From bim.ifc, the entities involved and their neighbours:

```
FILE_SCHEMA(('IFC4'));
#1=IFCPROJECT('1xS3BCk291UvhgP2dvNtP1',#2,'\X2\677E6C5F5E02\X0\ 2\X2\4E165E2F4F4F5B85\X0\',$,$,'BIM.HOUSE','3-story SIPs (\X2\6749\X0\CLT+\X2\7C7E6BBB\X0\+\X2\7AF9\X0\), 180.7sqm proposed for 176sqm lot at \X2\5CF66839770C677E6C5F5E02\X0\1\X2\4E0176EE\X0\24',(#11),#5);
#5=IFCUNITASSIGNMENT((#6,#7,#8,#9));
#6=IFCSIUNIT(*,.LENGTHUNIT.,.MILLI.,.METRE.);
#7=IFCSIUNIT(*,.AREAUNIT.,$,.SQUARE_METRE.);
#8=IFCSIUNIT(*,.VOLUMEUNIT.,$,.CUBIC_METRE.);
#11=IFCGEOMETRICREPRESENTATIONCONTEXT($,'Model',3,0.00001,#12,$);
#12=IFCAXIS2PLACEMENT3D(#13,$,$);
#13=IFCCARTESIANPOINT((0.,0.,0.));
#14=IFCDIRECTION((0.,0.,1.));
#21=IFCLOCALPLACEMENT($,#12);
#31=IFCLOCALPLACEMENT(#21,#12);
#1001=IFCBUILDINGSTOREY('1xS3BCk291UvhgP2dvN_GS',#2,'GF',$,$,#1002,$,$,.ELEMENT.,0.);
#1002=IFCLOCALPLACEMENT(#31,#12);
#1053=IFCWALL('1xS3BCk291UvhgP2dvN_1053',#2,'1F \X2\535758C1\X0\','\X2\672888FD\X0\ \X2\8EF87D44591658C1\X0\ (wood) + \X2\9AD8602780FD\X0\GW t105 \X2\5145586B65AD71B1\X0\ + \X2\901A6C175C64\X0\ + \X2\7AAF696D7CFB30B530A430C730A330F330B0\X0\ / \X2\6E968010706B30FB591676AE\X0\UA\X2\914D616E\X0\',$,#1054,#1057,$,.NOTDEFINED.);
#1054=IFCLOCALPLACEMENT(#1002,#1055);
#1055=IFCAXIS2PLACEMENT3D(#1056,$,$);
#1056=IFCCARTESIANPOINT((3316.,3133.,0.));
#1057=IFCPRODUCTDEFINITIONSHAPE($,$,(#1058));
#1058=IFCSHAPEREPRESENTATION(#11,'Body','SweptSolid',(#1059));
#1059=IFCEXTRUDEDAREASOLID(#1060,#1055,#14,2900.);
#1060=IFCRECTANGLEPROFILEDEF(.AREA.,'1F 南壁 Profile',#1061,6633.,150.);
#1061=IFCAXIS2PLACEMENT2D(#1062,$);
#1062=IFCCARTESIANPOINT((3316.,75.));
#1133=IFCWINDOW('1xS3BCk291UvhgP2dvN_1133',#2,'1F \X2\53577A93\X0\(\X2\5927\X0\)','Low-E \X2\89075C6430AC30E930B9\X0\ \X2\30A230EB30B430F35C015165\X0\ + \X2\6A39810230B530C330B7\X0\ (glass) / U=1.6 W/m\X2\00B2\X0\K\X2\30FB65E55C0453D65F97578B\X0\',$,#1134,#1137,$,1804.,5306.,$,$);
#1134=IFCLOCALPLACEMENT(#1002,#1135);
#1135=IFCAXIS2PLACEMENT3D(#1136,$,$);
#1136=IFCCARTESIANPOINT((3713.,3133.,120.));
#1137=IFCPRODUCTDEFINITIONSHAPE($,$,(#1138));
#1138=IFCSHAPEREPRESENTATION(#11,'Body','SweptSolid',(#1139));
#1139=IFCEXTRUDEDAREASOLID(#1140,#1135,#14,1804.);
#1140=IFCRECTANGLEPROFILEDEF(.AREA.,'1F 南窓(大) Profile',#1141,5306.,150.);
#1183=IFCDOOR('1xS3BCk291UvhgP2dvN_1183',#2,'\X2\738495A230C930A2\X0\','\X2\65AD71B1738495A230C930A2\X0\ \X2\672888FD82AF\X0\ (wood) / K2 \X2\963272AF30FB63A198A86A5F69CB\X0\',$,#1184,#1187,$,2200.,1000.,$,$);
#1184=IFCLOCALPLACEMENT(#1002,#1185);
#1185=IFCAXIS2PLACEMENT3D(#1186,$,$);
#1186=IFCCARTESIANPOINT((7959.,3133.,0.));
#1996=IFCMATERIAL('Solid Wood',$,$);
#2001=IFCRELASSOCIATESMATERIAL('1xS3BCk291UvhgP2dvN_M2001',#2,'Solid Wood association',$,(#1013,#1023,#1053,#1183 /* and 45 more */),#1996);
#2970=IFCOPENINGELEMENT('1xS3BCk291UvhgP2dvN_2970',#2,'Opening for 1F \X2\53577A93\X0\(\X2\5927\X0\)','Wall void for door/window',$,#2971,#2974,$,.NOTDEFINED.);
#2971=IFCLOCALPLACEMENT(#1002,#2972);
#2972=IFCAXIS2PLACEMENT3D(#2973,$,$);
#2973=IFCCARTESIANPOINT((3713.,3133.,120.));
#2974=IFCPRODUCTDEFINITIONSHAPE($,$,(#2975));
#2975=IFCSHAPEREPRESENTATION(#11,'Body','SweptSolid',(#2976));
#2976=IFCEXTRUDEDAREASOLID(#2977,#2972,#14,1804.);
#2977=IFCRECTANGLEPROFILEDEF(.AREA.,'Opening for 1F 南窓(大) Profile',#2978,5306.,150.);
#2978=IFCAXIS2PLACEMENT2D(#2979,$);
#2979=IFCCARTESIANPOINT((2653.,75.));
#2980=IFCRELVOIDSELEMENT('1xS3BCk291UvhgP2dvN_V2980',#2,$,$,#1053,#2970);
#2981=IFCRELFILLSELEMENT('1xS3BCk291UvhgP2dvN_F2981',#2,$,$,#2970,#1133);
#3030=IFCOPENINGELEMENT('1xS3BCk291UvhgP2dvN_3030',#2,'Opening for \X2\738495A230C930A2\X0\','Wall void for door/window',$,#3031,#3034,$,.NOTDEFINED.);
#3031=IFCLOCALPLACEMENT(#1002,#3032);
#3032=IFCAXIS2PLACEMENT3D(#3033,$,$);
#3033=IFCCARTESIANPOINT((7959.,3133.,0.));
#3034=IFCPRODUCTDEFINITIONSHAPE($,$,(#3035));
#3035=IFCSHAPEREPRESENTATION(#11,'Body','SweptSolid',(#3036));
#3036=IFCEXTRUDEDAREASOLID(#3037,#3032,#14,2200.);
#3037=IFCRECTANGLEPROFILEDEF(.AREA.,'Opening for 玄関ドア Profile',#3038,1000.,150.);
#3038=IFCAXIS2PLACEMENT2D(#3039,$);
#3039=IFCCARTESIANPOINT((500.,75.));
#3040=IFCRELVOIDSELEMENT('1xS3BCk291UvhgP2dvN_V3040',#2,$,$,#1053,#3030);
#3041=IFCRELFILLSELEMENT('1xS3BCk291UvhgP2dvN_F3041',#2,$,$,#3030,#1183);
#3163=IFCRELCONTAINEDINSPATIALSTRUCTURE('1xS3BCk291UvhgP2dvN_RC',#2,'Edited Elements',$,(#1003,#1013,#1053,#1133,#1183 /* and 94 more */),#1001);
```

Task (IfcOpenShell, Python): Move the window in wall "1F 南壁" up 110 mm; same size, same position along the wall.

```python
import numpy as np
import ifcopenshell
import ifcopenshell.api.geometry
import ifcopenshell.util.placement
import ifcopenshell.util.unit

model = ifcopenshell.open("bim.ifc")
unit_scale = ifcopenshell.util.unit.calculate_unit_scale(model)

window = model.by_id(1133)
opening = window.FillsVoids[0].RelatingOpeningElement
dz = 0.11 / unit_scale

shift = np.array([0.0, 0.0, dz])
# The window is not placed relative to its opening, so move both.
for product in (opening, window):
    matrix = ifcopenshell.util.placement.get_local_placement(product.ObjectPlacement)
    matrix[:3, 3] += shift
    ifcopenshell.api.geometry.edit_object_placement(model, product=product, matrix=matrix, is_si=False)

print(f"moved by {dz * unit_scale:+.3f} m")

model.write("bim_rev.ifc")
```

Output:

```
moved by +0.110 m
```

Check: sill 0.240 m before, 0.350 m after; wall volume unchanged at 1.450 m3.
